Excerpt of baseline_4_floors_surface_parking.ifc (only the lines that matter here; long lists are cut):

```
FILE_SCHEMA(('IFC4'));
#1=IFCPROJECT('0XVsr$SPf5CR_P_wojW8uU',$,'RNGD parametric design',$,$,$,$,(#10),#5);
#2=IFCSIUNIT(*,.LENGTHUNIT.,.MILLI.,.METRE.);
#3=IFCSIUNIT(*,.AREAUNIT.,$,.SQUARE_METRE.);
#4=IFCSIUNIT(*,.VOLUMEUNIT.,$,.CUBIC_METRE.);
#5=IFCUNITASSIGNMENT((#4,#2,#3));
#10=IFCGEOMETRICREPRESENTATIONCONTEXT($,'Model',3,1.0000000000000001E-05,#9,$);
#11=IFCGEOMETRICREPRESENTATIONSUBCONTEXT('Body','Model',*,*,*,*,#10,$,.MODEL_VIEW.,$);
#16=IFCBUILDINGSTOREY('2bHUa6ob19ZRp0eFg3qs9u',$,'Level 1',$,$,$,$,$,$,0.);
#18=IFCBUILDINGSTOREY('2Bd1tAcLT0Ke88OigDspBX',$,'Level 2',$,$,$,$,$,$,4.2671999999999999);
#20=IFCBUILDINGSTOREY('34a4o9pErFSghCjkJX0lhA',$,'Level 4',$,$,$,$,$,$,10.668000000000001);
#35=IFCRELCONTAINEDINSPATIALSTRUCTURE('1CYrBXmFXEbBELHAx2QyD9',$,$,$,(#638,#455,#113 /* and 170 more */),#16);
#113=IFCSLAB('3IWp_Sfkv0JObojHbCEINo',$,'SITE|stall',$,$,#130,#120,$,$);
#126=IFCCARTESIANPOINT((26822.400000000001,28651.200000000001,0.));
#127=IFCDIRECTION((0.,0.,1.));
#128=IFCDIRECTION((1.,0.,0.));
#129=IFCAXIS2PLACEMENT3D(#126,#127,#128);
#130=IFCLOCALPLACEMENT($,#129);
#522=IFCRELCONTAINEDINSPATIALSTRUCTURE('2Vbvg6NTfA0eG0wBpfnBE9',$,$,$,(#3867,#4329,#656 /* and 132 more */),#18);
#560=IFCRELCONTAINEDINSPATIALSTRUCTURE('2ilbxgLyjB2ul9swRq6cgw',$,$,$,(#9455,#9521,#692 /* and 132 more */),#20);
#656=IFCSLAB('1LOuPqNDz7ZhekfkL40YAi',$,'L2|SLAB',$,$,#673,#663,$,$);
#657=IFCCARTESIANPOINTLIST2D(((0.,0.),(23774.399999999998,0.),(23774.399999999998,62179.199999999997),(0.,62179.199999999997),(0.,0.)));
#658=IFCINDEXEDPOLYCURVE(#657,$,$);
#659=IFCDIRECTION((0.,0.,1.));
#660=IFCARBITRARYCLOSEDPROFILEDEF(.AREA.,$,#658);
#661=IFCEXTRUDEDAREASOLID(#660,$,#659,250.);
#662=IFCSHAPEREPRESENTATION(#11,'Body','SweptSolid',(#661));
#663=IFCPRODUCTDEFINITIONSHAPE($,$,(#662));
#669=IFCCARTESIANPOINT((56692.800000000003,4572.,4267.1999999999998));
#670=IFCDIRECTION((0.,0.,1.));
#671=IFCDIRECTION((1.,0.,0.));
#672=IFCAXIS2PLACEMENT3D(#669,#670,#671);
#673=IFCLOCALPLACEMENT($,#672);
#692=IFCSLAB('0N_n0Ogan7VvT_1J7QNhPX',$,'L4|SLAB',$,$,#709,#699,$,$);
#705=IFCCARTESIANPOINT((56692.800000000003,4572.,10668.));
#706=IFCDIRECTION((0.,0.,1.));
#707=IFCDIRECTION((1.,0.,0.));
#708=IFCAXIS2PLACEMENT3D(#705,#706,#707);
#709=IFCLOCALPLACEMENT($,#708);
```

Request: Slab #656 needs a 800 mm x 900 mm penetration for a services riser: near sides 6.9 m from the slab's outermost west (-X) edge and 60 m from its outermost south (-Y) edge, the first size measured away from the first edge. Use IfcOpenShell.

```python
import numpy as np
import ifcopenshell
import ifcopenshell.api.feature
import ifcopenshell.api.geometry
import ifcopenshell.api.root
import ifcopenshell.geom
import ifcopenshell.util.placement
import ifcopenshell.util.representation
import ifcopenshell.util.shape
import ifcopenshell.util.unit

model = ifcopenshell.open("baseline_4_floors_surface_parking.ifc")
unit_scale = ifcopenshell.util.unit.calculate_unit_scale(model)
settings = ifcopenshell.geom.settings()


def volume(element):
    """Net volume in cubic metres, openings subtracted."""
    shape = ifcopenshell.geom.create_shape(settings, element)
    return ifcopenshell.util.shape.get_volume(shape.geometry)


slab = model.by_guid("1LOuPqNDz7ZhekfkL40YAi")
before = volume(slab)

# Extent in the slab's own axes, in metres. The edges named are its -X and -Y sides.
slab_shape = ifcopenshell.geom.create_shape(settings, slab)
vertices = ifcopenshell.util.shape.get_vertices(slab_shape.geometry)
x_min, y_min, bottom = vertices.min(axis=0)
top = vertices[:, 2].max()

opening = ifcopenshell.api.root.create_entity(model, ifc_class="IfcOpeningElement", name="Services riser opening", predefined_type="OPENING")
context = ifcopenshell.util.representation.get_context(model, "Model", "Body", "MODEL_VIEW")
width, depth = 0.8, 0.9
outline = [(0.0, 0.0), (width, 0.0), (width, depth), (0.0, depth), (0.0, 0.0)]
# Overshoot both faces by 50 mm so the cut is clean.
shape = ifcopenshell.api.geometry.add_slab_representation(
    model, context=context, depth=top - bottom + 0.1, polyline=outline
)
ifcopenshell.api.geometry.assign_representation(model, product=opening, representation=shape)

matrix = ifcopenshell.util.placement.get_local_placement(slab.ObjectPlacement)
matrix[:, 3] = matrix @ np.append(np.array([x_min + 6.9, y_min + 60, bottom - 0.05]) / unit_scale, 1.0)
ifcopenshell.api.geometry.edit_object_placement(model, product=opening, matrix=matrix, is_si=False)
ifcopenshell.api.feature.add_feature(model, feature=opening, element=slab)

after = volume(slab)

print(f"slab volume {before:.3f} -> {after:.3f} m3")

model.write("baseline_4_floors_surface_parking_updated.ifc")
```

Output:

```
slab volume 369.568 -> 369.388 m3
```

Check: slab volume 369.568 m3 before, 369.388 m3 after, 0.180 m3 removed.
